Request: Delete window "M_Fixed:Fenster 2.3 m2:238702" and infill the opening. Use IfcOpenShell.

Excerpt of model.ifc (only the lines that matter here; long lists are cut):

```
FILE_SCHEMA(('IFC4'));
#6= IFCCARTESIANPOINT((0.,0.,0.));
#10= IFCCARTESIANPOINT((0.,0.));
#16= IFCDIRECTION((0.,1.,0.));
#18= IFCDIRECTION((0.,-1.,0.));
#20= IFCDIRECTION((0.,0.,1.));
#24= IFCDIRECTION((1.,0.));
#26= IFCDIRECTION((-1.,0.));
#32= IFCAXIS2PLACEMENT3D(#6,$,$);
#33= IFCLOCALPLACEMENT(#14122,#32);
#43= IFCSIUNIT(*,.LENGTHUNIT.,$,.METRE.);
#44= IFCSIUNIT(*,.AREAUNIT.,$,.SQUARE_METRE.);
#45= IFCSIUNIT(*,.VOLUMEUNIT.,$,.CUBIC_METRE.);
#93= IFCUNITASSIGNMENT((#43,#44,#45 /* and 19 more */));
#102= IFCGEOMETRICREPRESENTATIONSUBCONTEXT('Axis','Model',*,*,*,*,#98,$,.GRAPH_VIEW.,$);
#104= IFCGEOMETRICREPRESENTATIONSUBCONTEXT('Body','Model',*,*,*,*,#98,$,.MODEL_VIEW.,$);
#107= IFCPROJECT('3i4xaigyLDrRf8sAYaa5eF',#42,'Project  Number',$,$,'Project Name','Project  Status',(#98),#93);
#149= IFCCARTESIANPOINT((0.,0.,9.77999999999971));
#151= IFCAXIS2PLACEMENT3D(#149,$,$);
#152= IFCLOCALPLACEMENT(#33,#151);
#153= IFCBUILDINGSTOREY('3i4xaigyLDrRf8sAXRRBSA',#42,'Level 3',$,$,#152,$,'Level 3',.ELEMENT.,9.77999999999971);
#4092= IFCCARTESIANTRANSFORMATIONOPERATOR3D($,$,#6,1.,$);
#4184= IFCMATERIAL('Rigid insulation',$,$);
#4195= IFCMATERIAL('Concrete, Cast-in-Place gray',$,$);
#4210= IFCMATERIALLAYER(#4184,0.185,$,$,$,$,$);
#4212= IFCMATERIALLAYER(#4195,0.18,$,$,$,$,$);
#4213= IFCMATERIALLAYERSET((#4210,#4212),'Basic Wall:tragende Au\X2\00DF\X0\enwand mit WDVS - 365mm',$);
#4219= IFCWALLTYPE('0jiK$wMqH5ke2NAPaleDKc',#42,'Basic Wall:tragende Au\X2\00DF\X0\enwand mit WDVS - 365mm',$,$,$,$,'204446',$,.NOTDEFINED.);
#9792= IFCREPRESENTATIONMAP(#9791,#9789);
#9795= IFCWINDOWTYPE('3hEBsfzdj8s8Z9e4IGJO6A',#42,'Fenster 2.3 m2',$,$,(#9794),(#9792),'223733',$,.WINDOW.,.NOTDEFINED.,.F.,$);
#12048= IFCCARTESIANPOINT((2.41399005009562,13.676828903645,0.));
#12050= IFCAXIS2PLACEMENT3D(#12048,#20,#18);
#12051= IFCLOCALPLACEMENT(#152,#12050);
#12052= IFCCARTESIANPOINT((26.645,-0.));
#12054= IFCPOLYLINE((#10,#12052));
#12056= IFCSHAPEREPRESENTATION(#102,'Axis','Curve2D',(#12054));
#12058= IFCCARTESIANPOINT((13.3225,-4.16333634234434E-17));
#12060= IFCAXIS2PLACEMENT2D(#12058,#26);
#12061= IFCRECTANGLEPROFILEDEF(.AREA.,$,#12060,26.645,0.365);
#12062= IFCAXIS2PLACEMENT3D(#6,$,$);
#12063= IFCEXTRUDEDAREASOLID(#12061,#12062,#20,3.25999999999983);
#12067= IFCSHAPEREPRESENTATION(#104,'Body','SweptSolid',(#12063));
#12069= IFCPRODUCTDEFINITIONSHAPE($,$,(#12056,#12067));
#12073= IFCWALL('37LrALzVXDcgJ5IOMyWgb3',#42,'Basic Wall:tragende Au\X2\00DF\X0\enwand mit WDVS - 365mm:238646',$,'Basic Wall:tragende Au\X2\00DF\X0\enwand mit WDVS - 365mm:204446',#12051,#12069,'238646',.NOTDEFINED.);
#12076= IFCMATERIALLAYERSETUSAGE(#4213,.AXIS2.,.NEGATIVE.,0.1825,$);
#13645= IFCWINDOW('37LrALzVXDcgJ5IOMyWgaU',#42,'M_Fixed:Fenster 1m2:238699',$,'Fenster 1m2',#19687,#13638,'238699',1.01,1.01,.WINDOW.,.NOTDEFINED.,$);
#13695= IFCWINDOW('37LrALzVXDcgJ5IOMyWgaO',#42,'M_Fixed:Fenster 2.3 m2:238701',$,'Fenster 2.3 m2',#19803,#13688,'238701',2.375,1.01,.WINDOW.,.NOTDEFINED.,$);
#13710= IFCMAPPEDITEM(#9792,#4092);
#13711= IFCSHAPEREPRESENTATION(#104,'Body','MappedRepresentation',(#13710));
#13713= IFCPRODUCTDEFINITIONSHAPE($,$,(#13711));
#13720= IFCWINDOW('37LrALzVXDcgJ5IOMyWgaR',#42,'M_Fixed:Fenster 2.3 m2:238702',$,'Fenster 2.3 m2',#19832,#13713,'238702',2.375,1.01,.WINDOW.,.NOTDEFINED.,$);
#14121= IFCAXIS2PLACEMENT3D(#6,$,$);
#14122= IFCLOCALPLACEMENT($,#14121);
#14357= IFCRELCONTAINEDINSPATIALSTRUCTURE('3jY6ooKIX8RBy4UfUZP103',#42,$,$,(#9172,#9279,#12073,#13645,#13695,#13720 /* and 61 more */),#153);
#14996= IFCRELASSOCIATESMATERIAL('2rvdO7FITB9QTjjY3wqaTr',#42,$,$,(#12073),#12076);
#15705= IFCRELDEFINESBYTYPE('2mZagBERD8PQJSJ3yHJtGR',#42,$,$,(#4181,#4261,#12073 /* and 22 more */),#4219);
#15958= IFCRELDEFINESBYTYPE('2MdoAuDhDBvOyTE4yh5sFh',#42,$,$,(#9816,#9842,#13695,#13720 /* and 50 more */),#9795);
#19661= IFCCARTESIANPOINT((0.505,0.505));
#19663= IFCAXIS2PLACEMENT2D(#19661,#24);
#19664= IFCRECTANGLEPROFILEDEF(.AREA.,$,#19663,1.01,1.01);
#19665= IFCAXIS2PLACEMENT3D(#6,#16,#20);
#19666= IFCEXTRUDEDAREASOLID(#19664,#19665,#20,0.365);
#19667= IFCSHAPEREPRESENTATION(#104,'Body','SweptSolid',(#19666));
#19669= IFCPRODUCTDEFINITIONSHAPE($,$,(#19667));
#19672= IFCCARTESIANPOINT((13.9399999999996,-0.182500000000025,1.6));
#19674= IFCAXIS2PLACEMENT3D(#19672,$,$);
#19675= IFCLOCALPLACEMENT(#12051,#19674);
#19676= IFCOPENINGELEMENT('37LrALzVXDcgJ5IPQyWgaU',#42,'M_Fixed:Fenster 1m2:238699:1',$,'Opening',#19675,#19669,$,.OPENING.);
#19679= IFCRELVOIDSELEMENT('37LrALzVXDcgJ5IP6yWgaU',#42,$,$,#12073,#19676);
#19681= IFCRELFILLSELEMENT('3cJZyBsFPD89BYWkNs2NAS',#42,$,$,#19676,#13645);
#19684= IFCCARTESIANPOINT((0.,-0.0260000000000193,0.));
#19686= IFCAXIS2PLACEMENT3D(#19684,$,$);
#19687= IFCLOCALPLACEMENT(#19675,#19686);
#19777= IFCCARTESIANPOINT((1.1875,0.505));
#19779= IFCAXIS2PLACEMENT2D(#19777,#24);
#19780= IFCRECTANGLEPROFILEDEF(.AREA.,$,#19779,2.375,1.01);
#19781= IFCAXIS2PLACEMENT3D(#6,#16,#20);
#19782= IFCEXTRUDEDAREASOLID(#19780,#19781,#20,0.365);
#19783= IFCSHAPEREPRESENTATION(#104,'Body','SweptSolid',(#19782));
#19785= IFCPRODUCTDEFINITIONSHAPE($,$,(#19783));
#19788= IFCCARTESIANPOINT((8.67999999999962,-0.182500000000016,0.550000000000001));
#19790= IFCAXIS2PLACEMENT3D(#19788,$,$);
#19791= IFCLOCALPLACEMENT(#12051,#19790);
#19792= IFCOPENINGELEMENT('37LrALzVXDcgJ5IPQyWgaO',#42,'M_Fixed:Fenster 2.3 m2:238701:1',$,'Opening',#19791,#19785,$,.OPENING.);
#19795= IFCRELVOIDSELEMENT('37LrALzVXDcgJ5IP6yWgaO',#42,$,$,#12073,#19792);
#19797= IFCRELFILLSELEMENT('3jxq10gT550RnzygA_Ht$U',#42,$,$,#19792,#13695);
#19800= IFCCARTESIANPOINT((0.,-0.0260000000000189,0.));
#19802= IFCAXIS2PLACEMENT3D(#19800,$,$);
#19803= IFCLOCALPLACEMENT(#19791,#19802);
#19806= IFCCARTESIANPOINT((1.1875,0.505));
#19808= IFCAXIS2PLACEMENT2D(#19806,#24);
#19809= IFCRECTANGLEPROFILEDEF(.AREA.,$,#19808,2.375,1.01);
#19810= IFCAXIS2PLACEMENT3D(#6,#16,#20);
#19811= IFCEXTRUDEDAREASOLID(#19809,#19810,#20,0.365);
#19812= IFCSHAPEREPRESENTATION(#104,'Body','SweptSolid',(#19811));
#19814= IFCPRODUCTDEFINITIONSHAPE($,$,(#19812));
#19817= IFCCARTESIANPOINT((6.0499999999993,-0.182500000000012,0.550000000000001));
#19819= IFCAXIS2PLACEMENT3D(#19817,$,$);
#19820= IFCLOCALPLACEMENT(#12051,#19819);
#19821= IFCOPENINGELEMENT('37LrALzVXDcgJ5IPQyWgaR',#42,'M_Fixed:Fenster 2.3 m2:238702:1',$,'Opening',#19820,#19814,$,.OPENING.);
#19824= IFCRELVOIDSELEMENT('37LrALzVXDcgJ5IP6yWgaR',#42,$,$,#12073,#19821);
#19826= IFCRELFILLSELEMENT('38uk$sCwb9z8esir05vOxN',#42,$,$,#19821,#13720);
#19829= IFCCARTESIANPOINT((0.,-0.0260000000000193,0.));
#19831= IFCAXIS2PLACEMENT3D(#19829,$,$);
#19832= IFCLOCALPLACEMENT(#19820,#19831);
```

```python
import ifcopenshell
import ifcopenshell.api.feature
import ifcopenshell.api.root
import ifcopenshell.geom
import ifcopenshell.util.shape

model = ifcopenshell.open("model.ifc")
settings = ifcopenshell.geom.settings()


def volume(element):
    """Net volume in cubic metres, openings subtracted."""
    shape = ifcopenshell.geom.create_shape(settings, element)
    return ifcopenshell.util.shape.get_volume(shape.geometry)


window = model.by_guid("37LrALzVXDcgJ5IOMyWgaR")
opening = window.FillsVoids[0].RelatingOpeningElement
wall = opening.VoidsElements[0].RelatingBuildingElement
before = volume(wall)

ifcopenshell.api.root.remove_product(model, product=window)
ifcopenshell.api.feature.remove_feature(model, feature=opening)

after = volume(wall)

print(f"wall volume {before:.3f} -> {after:.3f} m3")

model.write("model_updated.ifc")
```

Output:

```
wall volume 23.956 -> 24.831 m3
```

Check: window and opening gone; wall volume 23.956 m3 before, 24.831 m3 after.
